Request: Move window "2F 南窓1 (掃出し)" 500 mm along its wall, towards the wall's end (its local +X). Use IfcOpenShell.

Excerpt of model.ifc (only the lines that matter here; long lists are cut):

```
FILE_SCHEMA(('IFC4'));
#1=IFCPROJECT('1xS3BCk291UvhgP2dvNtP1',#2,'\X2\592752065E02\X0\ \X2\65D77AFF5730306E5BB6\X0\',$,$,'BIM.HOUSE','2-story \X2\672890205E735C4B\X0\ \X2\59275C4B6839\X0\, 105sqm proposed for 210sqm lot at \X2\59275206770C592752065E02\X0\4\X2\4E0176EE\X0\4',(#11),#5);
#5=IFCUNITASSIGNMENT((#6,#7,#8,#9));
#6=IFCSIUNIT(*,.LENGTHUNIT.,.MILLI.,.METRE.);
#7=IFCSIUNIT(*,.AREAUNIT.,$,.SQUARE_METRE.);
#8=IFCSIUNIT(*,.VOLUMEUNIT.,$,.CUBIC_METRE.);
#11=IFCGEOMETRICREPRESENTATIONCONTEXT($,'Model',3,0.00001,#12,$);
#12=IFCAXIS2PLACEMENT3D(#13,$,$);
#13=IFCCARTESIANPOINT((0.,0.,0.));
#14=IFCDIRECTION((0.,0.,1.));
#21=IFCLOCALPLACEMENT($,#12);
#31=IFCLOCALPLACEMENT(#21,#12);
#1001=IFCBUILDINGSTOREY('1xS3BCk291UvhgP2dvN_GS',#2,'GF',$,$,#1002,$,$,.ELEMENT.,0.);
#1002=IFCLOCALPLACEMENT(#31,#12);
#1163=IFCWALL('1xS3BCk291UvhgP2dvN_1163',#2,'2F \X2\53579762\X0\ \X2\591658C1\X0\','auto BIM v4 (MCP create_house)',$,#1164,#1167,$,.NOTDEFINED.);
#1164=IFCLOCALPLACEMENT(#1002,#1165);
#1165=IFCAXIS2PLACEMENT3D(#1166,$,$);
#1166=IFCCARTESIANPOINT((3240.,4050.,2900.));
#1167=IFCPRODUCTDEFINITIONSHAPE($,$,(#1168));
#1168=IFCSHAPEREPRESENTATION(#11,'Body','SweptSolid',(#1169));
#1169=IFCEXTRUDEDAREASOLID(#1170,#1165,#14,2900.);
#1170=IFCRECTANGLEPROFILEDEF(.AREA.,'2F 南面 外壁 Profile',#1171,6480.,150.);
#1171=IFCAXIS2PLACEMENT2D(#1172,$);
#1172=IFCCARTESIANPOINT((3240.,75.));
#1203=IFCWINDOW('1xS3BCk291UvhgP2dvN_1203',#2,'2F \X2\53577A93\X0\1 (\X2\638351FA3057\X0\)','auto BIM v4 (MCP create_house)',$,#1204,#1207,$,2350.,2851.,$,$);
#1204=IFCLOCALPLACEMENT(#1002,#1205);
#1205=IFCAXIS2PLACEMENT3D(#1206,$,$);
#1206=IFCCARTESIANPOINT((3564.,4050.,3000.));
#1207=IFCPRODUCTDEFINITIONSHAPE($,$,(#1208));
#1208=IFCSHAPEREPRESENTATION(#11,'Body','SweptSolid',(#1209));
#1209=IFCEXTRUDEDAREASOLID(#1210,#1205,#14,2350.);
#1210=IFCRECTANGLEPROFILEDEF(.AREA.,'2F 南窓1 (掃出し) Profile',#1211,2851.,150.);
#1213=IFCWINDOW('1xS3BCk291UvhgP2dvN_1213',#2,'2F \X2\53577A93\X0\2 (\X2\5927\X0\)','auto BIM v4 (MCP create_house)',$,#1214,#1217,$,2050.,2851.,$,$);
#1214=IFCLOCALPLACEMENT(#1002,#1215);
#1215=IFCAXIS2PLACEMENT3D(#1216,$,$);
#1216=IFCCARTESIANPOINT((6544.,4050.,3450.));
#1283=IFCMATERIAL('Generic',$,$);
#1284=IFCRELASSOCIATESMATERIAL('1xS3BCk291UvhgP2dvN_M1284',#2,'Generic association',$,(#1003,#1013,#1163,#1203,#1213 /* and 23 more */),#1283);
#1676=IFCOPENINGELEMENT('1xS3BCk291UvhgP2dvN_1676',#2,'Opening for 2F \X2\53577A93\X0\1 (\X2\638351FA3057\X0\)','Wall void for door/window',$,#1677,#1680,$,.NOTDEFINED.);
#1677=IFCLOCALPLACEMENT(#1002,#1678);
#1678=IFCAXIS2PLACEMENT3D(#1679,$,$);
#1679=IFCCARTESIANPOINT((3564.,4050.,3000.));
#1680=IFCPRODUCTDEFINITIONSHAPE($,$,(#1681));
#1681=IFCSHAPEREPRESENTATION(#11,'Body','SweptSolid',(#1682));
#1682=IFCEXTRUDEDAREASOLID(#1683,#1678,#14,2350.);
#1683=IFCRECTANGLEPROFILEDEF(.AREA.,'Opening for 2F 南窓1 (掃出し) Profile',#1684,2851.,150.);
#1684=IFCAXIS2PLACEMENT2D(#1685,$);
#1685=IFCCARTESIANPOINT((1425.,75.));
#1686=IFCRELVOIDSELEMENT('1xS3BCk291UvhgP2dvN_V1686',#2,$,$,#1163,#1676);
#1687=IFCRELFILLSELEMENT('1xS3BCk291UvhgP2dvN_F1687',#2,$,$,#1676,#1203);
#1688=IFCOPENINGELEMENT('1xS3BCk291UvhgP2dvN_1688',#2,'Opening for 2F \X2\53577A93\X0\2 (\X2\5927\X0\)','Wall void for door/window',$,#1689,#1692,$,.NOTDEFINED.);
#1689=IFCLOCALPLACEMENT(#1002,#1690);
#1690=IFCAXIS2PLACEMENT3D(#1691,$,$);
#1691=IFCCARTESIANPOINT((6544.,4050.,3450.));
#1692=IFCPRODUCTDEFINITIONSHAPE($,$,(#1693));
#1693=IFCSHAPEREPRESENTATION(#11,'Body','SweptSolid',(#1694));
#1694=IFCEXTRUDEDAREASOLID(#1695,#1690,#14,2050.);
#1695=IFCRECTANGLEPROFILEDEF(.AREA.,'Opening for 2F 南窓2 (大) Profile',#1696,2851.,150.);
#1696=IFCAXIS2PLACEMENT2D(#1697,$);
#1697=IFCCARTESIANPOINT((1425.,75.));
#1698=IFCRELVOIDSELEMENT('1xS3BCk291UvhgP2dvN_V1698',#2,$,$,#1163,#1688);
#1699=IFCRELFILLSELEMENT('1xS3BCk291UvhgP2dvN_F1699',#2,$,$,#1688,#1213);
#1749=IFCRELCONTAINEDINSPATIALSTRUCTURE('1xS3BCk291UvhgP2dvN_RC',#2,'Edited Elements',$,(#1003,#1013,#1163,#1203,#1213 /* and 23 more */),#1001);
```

```python
import ifcopenshell
import ifcopenshell.api.geometry
import ifcopenshell.util.placement
import ifcopenshell.util.unit

model = ifcopenshell.open("model.ifc")
unit_scale = ifcopenshell.util.unit.calculate_unit_scale(model)

window = model.by_id(1203)
opening = window.FillsVoids[0].RelatingOpeningElement
wall = opening.VoidsElements[0].RelatingBuildingElement

wall_matrix = ifcopenshell.util.placement.get_local_placement(wall.ObjectPlacement)
shift = wall_matrix[:3, 0] * 0.5 / unit_scale
before = ifcopenshell.util.placement.get_local_placement(window.ObjectPlacement)[:3, 3].copy()

# The window is not placed relative to its opening, so move both.
for product in (opening, window):
    matrix = ifcopenshell.util.placement.get_local_placement(product.ObjectPlacement)
    matrix[:3, 3] += shift
    ifcopenshell.api.geometry.edit_object_placement(model, product=product, matrix=matrix, is_si=False)

after = ifcopenshell.util.placement.get_local_placement(window.ObjectPlacement)[:3, 3]
print("window moved by", (after - before).round(3) + 0.0)

model.write("model-out.ifc")
```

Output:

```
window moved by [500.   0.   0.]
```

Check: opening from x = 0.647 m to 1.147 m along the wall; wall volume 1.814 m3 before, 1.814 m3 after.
